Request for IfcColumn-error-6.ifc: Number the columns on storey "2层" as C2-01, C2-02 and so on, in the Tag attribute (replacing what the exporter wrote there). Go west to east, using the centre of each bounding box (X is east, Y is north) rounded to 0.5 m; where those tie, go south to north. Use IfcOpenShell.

First a look at what the model holds.

```python
import ifcopenshell
import ifcopenshell.util.element
import ifcopenshell.util.placement

model = ifcopenshell.open("IfcColumn-error-6.ifc")
print(model.schema)
storey = next(s for s in model.by_type("IfcBuildingStorey") if s.Name == "2层")
columns = [e for e in ifcopenshell.util.element.get_decomposition(storey) if e.is_a("IfcColumn")]
for e in sorted(columns, key=lambda e: e.id()):
    origin = ifcopenshell.util.placement.get_local_placement(e.ObjectPlacement)[:3, 3]
    print(e.id(), e.Tag, e.Name, origin.round(2) + 0.0, sep=" | ")
```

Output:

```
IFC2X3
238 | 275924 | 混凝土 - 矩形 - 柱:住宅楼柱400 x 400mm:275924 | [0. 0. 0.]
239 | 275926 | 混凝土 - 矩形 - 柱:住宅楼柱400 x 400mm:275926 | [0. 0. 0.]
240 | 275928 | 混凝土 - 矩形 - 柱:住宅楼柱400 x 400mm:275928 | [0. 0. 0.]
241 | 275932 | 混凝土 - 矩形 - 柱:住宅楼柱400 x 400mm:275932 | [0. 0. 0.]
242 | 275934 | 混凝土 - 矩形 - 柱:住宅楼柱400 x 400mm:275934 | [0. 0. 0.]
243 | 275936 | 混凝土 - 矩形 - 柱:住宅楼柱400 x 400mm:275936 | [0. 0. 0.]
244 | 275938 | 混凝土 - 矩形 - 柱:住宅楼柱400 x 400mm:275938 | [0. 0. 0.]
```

```python
import ifcopenshell
import ifcopenshell.geom
import ifcopenshell.util.element
import ifcopenshell.util.shape

model = ifcopenshell.open("IfcColumn-error-6.ifc")
settings = ifcopenshell.geom.settings()
settings.set("use-world-coords", True)


def centre(element):
    shape = ifcopenshell.geom.create_shape(settings, element)
    return ifcopenshell.util.shape.get_bbox_centroid(shape.geometry)


storey = next(s for s in model.by_type("IfcBuildingStorey") if s.Name == "2层")
columns = [e for e in ifcopenshell.util.element.get_decomposition(storey) if e.is_a("IfcColumn")]

# Insertion points can sit at a corner or the storey origin, so sort by the geometry (in metres).
centres = {e: centre(e) for e in columns}
columns.sort(key=lambda e: (round(centres[e][0] / 0.5), centres[e][1]))

for i, e in enumerate(columns, start=1):
    number = f"C2-{i:02d}"
    e.Tag = number
    print(e.id(), number)

model.write("IfcColumn-error-6-out.ifc")
```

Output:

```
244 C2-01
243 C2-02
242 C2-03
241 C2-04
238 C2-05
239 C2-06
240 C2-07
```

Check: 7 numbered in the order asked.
